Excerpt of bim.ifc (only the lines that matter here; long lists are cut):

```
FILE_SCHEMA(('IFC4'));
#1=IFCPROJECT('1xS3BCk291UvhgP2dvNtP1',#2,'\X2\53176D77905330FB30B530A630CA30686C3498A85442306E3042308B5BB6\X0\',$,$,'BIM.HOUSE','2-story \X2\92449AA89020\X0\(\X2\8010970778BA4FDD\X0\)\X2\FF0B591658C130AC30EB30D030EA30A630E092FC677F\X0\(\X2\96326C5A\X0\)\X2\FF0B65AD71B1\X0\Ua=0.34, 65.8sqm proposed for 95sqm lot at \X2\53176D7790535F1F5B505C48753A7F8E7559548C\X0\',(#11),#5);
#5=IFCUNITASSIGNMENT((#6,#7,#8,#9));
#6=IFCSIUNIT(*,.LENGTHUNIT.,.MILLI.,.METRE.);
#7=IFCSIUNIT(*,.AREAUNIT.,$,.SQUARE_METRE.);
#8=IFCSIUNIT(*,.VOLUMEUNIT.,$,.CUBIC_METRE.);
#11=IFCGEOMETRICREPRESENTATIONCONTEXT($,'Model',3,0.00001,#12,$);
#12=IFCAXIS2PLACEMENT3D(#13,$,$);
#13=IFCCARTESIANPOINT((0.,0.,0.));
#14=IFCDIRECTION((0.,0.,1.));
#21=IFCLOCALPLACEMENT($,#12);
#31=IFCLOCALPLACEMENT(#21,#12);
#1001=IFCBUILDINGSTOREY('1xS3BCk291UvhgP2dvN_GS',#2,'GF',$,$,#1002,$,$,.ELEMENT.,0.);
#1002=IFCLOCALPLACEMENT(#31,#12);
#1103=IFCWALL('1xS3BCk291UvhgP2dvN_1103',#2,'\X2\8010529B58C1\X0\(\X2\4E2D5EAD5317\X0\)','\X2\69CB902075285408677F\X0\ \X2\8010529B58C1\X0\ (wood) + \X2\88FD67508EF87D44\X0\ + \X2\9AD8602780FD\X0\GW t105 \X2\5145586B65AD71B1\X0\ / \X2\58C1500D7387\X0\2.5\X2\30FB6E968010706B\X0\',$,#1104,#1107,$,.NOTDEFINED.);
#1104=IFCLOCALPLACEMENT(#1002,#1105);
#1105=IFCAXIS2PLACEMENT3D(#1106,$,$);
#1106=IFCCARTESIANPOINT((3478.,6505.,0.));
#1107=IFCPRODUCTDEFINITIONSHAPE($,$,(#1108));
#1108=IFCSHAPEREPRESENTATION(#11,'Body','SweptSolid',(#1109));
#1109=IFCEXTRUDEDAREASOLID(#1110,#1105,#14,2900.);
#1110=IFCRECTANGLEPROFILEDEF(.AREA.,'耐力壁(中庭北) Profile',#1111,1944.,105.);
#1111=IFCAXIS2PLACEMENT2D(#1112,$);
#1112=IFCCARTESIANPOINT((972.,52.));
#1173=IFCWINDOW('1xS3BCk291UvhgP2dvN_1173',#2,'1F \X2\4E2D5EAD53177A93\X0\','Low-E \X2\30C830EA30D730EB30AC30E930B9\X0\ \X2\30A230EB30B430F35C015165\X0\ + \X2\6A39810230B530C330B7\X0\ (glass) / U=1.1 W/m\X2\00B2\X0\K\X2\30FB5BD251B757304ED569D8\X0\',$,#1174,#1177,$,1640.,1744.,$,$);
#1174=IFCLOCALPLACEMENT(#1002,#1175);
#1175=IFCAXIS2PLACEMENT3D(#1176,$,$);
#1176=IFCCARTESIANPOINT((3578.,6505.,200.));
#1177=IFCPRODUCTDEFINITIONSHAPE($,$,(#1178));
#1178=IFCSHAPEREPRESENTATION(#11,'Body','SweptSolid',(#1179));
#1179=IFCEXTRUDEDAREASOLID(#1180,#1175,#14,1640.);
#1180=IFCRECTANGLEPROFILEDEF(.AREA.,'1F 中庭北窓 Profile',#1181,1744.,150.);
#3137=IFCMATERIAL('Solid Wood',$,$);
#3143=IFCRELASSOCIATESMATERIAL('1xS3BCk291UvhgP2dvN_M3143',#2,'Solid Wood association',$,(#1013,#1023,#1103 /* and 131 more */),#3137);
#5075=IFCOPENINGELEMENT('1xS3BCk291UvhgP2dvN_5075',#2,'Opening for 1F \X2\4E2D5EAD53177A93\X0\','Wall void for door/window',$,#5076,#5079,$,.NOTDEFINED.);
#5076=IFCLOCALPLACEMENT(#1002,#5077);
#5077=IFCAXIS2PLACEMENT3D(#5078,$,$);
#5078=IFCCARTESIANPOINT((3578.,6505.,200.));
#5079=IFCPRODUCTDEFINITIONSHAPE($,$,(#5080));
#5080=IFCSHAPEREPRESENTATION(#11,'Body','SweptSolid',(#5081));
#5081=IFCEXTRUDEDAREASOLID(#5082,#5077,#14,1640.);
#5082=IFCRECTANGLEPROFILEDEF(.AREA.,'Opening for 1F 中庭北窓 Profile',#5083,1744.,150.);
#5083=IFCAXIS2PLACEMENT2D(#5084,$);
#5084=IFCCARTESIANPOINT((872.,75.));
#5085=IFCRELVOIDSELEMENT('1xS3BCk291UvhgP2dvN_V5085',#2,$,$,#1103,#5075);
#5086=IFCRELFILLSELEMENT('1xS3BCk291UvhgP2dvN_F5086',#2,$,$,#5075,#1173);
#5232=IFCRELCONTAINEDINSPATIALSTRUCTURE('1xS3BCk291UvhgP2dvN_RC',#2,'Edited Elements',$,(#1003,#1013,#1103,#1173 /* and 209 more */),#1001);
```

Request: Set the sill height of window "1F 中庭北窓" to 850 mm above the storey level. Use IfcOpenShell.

```python
import numpy as np
import ifcopenshell
import ifcopenshell.api.geometry
import ifcopenshell.geom
import ifcopenshell.util.element
import ifcopenshell.util.placement
import ifcopenshell.util.shape
import ifcopenshell.util.unit

model = ifcopenshell.open("bim.ifc")
unit_scale = ifcopenshell.util.unit.calculate_unit_scale(model)

window = model.by_id(1173)
opening = window.FillsVoids[0].RelatingOpeningElement
storey = ifcopenshell.util.element.get_container(window, ifc_class="IfcBuildingStorey")
level = ifcopenshell.util.placement.get_local_placement(storey.ObjectPlacement)[2, 3]

# The opening's origin need not be at the sill, so measure its lowest point.
shape = ifcopenshell.geom.create_shape(ifcopenshell.geom.settings(), opening)
bottom = ifcopenshell.util.shape.get_shape_bottom_elevation(shape, shape.geometry) / unit_scale
dz = level + 0.85 / unit_scale - bottom

shift = np.array([0.0, 0.0, dz])
# The window is not placed relative to its opening, so move both.
for product in (opening, window):
    matrix = ifcopenshell.util.placement.get_local_placement(product.ObjectPlacement)
    matrix[:3, 3] += shift
    ifcopenshell.api.geometry.edit_object_placement(model, product=product, matrix=matrix, is_si=False)

print(f"moved by {dz * unit_scale:+.3f} m")

model.write("bim-out.ifc")
```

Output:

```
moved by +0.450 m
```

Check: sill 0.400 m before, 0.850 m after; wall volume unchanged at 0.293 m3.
